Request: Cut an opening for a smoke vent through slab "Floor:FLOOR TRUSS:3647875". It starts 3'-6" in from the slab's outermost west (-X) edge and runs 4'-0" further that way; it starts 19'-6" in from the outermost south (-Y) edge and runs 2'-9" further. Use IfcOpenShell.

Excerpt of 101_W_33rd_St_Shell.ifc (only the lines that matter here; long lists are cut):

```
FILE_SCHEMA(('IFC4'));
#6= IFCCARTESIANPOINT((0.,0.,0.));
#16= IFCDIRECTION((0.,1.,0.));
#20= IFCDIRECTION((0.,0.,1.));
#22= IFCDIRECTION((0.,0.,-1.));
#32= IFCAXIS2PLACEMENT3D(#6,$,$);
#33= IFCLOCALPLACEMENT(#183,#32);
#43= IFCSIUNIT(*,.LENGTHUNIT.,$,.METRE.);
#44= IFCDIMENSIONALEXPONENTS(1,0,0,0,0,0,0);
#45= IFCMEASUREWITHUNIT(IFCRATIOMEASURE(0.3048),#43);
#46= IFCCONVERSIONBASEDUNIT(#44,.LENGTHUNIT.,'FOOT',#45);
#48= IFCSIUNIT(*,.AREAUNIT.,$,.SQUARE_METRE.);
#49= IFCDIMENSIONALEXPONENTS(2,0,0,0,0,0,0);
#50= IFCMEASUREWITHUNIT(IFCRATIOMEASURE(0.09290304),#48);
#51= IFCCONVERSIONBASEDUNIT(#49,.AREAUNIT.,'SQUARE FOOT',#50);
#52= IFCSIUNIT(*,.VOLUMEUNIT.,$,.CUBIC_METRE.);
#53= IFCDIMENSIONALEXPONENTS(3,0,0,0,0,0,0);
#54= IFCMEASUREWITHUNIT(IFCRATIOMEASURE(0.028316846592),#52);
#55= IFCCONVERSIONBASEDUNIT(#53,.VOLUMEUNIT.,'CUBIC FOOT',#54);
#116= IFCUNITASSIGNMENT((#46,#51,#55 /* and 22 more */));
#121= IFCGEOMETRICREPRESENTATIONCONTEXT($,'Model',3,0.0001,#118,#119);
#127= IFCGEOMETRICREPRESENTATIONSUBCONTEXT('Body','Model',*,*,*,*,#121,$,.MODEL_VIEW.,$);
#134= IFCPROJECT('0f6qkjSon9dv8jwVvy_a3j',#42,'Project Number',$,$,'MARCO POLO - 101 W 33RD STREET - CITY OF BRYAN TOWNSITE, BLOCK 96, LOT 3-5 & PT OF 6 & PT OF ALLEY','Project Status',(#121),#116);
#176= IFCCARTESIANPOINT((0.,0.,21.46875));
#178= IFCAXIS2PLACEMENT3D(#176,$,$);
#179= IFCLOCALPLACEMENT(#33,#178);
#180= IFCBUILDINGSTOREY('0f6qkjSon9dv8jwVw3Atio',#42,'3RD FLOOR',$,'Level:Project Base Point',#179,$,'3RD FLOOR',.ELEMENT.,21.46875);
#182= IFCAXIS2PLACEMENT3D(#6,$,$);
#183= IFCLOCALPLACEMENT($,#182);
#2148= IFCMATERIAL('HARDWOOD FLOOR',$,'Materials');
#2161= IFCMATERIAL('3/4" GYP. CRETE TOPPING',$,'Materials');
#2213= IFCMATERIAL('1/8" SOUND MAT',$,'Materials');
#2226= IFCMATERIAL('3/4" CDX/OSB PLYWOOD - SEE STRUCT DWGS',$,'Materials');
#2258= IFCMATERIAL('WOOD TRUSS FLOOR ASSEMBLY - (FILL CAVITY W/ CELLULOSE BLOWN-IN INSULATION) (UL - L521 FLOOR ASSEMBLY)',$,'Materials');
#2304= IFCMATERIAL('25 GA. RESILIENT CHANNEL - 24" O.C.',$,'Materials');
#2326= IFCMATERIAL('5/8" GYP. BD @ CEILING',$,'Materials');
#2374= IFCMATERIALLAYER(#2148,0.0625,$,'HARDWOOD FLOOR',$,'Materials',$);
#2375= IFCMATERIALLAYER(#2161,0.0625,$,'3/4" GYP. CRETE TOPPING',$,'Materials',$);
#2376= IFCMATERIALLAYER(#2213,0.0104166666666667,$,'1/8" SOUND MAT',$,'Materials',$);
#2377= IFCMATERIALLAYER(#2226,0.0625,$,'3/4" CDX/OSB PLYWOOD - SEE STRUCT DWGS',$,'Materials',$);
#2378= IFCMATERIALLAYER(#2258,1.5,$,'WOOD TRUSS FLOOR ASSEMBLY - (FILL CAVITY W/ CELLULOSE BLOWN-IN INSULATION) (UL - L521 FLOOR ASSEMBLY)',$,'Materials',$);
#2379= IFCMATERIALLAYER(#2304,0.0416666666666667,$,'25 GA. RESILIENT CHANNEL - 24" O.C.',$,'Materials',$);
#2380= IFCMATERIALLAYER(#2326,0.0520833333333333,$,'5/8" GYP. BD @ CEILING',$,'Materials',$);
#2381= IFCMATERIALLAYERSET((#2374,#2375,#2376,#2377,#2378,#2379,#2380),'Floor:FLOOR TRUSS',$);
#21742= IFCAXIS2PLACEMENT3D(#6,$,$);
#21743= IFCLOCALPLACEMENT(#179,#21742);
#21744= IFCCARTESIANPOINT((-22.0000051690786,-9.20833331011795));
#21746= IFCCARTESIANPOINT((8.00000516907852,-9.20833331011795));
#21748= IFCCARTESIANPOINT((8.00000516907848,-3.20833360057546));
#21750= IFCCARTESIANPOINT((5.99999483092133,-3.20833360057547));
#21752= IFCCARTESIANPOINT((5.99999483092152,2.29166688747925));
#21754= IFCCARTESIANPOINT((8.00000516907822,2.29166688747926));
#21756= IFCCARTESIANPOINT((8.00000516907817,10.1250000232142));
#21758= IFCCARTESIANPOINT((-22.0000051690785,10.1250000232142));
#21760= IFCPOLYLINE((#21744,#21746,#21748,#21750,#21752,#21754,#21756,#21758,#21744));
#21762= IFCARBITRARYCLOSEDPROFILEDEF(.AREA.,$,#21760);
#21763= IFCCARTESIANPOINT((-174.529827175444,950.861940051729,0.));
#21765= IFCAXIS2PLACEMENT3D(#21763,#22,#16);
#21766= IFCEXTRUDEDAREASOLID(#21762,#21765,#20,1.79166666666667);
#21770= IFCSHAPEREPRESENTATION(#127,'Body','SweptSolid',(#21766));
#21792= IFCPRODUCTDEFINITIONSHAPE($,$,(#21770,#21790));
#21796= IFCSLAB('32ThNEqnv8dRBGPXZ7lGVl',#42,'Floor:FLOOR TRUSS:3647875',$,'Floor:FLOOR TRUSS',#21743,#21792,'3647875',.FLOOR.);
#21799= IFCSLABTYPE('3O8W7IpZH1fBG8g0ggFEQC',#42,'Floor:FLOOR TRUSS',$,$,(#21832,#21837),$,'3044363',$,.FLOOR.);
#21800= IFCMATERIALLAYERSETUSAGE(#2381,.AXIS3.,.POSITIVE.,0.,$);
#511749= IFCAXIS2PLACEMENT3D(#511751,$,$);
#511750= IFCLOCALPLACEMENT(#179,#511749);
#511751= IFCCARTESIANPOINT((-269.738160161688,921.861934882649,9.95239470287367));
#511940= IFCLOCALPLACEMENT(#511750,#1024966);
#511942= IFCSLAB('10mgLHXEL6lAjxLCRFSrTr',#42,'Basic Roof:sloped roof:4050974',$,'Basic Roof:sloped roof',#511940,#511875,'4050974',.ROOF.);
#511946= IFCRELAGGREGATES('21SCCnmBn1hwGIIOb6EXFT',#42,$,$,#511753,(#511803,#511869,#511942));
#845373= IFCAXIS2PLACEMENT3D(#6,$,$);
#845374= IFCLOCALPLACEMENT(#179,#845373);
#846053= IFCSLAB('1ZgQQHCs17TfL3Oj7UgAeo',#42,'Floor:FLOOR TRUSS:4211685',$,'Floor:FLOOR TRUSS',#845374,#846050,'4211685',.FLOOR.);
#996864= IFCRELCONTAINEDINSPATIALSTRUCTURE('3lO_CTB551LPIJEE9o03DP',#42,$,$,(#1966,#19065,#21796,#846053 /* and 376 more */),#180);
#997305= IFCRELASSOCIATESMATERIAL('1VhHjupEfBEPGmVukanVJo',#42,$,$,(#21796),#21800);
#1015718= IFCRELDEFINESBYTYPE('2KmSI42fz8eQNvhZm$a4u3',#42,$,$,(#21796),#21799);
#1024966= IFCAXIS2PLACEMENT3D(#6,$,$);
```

```python
import numpy as np
import ifcopenshell
import ifcopenshell.api.feature
import ifcopenshell.api.geometry
import ifcopenshell.api.root
import ifcopenshell.geom
import ifcopenshell.util.placement
import ifcopenshell.util.representation
import ifcopenshell.util.shape
import ifcopenshell.util.unit

model = ifcopenshell.open("101_W_33rd_St_Shell.ifc")
unit_scale = ifcopenshell.util.unit.calculate_unit_scale(model)
settings = ifcopenshell.geom.settings()


def volume(element):
    """Net volume in cubic metres, openings subtracted."""
    shape = ifcopenshell.geom.create_shape(settings, element)
    return ifcopenshell.util.shape.get_volume(shape.geometry)


slab = model.by_id(21796)
before = volume(slab)

# Extent in the slab's own axes, in metres. The edges named are its -X and -Y sides.
slab_shape = ifcopenshell.geom.create_shape(settings, slab)
vertices = ifcopenshell.util.shape.get_vertices(slab_shape.geometry)
x_min, y_min, bottom = vertices.min(axis=0)
top = vertices[:, 2].max()

opening = ifcopenshell.api.root.create_entity(model, ifc_class="IfcOpeningElement", name="Smoke vent opening", predefined_type="OPENING")
context = ifcopenshell.util.representation.get_context(model, "Model", "Body", "MODEL_VIEW")
width, depth = 1.2192, 0.8382
outline = [(0.0, 0.0), (width, 0.0), (width, depth), (0.0, depth), (0.0, 0.0)]
# Overshoot both faces by 50 mm so the cut is clean.
shape = ifcopenshell.api.geometry.add_slab_representation(
    model, context=context, depth=top - bottom + 0.1, polyline=outline
)
ifcopenshell.api.geometry.assign_representation(model, product=opening, representation=shape)

matrix = ifcopenshell.util.placement.get_local_placement(slab.ObjectPlacement)
matrix[:, 3] = matrix @ np.append(np.array([x_min + 1.0668, y_min + 5.9436, bottom - 0.05]) / unit_scale, 1.0)
ifcopenshell.api.geometry.edit_object_placement(model, product=opening, matrix=matrix, is_si=False)
ifcopenshell.api.feature.add_feature(model, feature=opening, element=slab)

after = volume(slab)

print(f"slab volume {before:.3f} -> {after:.3f} m3")

model.write("101_W_33rd_St_Shell_edited.ifc")
```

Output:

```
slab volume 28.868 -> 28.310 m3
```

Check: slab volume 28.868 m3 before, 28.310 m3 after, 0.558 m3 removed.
